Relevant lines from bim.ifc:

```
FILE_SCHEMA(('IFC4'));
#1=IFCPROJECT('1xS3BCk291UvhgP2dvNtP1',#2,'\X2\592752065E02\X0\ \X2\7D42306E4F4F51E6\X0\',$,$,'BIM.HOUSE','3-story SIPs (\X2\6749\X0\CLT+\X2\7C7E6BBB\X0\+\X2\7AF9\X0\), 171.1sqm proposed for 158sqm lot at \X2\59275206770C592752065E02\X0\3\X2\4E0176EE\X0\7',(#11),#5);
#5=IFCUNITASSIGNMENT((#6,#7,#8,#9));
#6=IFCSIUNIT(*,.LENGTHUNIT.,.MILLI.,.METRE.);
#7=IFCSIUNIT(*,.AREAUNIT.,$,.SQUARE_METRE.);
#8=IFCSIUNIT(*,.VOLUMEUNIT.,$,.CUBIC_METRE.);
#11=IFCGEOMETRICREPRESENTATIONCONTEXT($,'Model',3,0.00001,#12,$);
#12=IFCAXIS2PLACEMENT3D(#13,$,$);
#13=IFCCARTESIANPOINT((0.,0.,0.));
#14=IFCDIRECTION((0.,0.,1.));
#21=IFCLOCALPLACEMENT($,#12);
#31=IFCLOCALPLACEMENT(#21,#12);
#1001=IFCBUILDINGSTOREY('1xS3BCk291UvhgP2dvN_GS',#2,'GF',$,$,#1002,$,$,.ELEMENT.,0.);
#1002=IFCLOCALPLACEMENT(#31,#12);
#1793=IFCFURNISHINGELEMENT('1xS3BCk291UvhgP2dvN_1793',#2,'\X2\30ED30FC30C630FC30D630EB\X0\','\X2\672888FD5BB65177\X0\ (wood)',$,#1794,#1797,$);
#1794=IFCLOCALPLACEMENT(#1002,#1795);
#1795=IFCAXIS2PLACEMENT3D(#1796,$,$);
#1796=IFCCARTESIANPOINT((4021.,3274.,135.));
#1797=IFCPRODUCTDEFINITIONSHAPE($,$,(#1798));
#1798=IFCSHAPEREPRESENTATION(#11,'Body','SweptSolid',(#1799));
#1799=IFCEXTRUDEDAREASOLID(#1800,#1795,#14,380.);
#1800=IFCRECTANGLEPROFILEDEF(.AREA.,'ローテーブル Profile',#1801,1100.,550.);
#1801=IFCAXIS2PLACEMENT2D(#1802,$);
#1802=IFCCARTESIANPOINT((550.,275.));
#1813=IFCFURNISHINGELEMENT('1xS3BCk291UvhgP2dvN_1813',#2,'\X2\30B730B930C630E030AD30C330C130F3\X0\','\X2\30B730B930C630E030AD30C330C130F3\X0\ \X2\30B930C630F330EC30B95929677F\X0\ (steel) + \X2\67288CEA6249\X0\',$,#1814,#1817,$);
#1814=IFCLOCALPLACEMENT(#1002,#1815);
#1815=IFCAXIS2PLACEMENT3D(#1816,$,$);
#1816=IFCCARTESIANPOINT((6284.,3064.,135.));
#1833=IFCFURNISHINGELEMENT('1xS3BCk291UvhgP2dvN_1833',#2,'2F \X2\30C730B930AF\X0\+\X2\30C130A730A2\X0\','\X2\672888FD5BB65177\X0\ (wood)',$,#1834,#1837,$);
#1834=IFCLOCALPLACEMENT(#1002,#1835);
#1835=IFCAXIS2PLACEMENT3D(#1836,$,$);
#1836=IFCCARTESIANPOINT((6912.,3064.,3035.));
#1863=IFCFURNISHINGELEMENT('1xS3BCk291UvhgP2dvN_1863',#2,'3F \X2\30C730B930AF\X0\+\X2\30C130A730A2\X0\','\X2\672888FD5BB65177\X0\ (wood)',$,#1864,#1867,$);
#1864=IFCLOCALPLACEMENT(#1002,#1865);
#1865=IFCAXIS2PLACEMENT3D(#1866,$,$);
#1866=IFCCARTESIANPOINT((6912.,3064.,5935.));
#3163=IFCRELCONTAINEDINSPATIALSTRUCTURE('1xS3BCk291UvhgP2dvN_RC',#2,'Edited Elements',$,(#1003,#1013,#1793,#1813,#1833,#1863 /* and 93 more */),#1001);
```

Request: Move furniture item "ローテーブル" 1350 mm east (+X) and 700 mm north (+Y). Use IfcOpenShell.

```python
import ifcopenshell
import ifcopenshell.api.geometry
import ifcopenshell.util.placement
import ifcopenshell.util.unit

model = ifcopenshell.open("bim.ifc")
unit_scale = ifcopenshell.util.unit.calculate_unit_scale(model)

item = model.by_guid("1xS3BCk291UvhgP2dvN_1793")
matrix = ifcopenshell.util.placement.get_local_placement(item.ObjectPlacement)
matrix[0, 3] += 1.35 / unit_scale
matrix[1, 3] += 0.7 / unit_scale
ifcopenshell.api.geometry.edit_object_placement(model, product=item, matrix=matrix, is_si=False)

print(ifcopenshell.util.placement.get_local_placement(item.ObjectPlacement).round(3) + 0.0)

model.write("bim_rev.ifc")
```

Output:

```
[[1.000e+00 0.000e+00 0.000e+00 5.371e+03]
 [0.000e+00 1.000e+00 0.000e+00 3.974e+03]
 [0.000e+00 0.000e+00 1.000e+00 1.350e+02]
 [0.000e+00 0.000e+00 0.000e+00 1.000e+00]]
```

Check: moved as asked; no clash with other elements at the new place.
